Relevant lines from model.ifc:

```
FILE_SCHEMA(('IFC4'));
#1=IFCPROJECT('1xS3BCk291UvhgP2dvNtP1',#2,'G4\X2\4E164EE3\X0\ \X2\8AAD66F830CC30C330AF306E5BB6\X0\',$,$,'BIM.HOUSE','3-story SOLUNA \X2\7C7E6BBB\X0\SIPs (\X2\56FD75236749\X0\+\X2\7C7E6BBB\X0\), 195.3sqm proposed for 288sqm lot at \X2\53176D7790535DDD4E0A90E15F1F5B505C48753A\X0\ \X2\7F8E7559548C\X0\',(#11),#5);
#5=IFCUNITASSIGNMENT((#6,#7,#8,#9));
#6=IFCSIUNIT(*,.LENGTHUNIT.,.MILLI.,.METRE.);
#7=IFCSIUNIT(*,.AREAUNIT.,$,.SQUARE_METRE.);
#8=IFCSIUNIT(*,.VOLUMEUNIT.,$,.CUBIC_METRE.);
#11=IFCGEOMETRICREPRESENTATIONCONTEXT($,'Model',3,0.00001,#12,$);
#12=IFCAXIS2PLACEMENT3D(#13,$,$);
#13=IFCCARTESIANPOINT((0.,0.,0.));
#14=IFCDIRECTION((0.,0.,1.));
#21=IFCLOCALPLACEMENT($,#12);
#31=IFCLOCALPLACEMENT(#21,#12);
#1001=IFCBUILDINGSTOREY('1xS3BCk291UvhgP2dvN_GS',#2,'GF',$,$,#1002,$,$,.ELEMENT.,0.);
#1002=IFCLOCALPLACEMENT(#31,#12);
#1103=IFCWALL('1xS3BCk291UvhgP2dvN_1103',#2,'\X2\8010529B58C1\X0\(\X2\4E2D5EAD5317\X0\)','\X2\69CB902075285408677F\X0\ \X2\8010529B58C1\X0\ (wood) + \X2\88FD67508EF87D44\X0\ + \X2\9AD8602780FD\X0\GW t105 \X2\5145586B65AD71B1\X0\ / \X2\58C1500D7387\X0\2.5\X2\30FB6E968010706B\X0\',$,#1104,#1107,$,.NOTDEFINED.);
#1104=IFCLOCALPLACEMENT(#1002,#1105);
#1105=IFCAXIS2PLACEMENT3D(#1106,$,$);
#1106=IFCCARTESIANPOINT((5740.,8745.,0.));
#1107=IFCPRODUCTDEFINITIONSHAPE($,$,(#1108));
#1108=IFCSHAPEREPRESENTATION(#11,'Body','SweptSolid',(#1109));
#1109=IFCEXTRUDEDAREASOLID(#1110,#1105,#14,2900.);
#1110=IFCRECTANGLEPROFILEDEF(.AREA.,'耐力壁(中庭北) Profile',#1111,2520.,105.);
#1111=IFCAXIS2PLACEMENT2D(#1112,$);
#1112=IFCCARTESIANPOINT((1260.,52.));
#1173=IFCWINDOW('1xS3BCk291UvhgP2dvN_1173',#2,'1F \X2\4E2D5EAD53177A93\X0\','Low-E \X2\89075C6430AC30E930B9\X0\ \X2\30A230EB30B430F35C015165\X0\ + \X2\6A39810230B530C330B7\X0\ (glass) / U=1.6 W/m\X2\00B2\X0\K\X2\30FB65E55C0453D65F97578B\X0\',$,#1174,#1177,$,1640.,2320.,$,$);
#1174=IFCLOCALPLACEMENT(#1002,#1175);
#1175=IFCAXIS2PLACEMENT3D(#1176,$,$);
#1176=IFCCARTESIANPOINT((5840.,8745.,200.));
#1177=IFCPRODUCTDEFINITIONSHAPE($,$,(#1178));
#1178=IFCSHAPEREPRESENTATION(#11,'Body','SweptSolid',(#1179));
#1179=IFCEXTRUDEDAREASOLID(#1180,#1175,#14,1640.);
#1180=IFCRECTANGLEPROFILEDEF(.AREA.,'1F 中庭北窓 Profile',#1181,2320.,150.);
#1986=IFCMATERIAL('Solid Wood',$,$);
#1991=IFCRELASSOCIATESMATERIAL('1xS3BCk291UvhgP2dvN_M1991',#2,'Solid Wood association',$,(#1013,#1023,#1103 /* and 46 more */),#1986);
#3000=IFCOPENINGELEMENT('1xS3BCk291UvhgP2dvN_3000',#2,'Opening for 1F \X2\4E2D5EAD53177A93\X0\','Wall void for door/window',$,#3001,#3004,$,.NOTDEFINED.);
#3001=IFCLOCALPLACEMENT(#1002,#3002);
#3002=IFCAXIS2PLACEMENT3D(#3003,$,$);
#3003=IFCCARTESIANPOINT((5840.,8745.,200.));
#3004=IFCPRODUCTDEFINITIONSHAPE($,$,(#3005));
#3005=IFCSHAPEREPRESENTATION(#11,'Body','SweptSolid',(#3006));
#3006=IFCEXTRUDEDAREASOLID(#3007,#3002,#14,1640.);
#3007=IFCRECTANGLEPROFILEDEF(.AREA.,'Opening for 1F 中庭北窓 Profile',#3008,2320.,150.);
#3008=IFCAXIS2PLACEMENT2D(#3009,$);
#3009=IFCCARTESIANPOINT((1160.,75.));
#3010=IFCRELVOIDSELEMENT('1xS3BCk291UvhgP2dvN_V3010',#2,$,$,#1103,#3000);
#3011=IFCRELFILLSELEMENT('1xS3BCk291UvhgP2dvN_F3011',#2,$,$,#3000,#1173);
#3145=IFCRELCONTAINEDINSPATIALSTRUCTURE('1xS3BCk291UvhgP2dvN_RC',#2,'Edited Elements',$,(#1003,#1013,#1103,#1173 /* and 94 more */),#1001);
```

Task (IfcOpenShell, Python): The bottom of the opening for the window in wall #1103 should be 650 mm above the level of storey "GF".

```python
import numpy as np
import ifcopenshell
import ifcopenshell.api.geometry
import ifcopenshell.geom
import ifcopenshell.util.element
import ifcopenshell.util.placement
import ifcopenshell.util.shape
import ifcopenshell.util.unit

model = ifcopenshell.open("model.ifc")
unit_scale = ifcopenshell.util.unit.calculate_unit_scale(model)

window = model.by_id(1173)
opening = window.FillsVoids[0].RelatingOpeningElement
storey = ifcopenshell.util.element.get_container(window, ifc_class="IfcBuildingStorey")
level = ifcopenshell.util.placement.get_local_placement(storey.ObjectPlacement)[2, 3]

# The opening's origin need not be at the sill, so measure its lowest point.
shape = ifcopenshell.geom.create_shape(ifcopenshell.geom.settings(), opening)
bottom = ifcopenshell.util.shape.get_shape_bottom_elevation(shape, shape.geometry) / unit_scale
dz = level + 650.0 - bottom

shift = np.array([0.0, 0.0, dz])
# The window is not placed relative to its opening, so move both.
for product in (opening, window):
    matrix = ifcopenshell.util.placement.get_local_placement(product.ObjectPlacement)
    matrix[:3, 3] += shift
    ifcopenshell.api.geometry.edit_object_placement(model, product=product, matrix=matrix, is_si=False)

print(f"moved by {dz * unit_scale:+.3f} m")

model.write("model_updated.ifc")
```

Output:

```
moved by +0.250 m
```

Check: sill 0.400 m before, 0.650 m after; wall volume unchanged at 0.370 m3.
